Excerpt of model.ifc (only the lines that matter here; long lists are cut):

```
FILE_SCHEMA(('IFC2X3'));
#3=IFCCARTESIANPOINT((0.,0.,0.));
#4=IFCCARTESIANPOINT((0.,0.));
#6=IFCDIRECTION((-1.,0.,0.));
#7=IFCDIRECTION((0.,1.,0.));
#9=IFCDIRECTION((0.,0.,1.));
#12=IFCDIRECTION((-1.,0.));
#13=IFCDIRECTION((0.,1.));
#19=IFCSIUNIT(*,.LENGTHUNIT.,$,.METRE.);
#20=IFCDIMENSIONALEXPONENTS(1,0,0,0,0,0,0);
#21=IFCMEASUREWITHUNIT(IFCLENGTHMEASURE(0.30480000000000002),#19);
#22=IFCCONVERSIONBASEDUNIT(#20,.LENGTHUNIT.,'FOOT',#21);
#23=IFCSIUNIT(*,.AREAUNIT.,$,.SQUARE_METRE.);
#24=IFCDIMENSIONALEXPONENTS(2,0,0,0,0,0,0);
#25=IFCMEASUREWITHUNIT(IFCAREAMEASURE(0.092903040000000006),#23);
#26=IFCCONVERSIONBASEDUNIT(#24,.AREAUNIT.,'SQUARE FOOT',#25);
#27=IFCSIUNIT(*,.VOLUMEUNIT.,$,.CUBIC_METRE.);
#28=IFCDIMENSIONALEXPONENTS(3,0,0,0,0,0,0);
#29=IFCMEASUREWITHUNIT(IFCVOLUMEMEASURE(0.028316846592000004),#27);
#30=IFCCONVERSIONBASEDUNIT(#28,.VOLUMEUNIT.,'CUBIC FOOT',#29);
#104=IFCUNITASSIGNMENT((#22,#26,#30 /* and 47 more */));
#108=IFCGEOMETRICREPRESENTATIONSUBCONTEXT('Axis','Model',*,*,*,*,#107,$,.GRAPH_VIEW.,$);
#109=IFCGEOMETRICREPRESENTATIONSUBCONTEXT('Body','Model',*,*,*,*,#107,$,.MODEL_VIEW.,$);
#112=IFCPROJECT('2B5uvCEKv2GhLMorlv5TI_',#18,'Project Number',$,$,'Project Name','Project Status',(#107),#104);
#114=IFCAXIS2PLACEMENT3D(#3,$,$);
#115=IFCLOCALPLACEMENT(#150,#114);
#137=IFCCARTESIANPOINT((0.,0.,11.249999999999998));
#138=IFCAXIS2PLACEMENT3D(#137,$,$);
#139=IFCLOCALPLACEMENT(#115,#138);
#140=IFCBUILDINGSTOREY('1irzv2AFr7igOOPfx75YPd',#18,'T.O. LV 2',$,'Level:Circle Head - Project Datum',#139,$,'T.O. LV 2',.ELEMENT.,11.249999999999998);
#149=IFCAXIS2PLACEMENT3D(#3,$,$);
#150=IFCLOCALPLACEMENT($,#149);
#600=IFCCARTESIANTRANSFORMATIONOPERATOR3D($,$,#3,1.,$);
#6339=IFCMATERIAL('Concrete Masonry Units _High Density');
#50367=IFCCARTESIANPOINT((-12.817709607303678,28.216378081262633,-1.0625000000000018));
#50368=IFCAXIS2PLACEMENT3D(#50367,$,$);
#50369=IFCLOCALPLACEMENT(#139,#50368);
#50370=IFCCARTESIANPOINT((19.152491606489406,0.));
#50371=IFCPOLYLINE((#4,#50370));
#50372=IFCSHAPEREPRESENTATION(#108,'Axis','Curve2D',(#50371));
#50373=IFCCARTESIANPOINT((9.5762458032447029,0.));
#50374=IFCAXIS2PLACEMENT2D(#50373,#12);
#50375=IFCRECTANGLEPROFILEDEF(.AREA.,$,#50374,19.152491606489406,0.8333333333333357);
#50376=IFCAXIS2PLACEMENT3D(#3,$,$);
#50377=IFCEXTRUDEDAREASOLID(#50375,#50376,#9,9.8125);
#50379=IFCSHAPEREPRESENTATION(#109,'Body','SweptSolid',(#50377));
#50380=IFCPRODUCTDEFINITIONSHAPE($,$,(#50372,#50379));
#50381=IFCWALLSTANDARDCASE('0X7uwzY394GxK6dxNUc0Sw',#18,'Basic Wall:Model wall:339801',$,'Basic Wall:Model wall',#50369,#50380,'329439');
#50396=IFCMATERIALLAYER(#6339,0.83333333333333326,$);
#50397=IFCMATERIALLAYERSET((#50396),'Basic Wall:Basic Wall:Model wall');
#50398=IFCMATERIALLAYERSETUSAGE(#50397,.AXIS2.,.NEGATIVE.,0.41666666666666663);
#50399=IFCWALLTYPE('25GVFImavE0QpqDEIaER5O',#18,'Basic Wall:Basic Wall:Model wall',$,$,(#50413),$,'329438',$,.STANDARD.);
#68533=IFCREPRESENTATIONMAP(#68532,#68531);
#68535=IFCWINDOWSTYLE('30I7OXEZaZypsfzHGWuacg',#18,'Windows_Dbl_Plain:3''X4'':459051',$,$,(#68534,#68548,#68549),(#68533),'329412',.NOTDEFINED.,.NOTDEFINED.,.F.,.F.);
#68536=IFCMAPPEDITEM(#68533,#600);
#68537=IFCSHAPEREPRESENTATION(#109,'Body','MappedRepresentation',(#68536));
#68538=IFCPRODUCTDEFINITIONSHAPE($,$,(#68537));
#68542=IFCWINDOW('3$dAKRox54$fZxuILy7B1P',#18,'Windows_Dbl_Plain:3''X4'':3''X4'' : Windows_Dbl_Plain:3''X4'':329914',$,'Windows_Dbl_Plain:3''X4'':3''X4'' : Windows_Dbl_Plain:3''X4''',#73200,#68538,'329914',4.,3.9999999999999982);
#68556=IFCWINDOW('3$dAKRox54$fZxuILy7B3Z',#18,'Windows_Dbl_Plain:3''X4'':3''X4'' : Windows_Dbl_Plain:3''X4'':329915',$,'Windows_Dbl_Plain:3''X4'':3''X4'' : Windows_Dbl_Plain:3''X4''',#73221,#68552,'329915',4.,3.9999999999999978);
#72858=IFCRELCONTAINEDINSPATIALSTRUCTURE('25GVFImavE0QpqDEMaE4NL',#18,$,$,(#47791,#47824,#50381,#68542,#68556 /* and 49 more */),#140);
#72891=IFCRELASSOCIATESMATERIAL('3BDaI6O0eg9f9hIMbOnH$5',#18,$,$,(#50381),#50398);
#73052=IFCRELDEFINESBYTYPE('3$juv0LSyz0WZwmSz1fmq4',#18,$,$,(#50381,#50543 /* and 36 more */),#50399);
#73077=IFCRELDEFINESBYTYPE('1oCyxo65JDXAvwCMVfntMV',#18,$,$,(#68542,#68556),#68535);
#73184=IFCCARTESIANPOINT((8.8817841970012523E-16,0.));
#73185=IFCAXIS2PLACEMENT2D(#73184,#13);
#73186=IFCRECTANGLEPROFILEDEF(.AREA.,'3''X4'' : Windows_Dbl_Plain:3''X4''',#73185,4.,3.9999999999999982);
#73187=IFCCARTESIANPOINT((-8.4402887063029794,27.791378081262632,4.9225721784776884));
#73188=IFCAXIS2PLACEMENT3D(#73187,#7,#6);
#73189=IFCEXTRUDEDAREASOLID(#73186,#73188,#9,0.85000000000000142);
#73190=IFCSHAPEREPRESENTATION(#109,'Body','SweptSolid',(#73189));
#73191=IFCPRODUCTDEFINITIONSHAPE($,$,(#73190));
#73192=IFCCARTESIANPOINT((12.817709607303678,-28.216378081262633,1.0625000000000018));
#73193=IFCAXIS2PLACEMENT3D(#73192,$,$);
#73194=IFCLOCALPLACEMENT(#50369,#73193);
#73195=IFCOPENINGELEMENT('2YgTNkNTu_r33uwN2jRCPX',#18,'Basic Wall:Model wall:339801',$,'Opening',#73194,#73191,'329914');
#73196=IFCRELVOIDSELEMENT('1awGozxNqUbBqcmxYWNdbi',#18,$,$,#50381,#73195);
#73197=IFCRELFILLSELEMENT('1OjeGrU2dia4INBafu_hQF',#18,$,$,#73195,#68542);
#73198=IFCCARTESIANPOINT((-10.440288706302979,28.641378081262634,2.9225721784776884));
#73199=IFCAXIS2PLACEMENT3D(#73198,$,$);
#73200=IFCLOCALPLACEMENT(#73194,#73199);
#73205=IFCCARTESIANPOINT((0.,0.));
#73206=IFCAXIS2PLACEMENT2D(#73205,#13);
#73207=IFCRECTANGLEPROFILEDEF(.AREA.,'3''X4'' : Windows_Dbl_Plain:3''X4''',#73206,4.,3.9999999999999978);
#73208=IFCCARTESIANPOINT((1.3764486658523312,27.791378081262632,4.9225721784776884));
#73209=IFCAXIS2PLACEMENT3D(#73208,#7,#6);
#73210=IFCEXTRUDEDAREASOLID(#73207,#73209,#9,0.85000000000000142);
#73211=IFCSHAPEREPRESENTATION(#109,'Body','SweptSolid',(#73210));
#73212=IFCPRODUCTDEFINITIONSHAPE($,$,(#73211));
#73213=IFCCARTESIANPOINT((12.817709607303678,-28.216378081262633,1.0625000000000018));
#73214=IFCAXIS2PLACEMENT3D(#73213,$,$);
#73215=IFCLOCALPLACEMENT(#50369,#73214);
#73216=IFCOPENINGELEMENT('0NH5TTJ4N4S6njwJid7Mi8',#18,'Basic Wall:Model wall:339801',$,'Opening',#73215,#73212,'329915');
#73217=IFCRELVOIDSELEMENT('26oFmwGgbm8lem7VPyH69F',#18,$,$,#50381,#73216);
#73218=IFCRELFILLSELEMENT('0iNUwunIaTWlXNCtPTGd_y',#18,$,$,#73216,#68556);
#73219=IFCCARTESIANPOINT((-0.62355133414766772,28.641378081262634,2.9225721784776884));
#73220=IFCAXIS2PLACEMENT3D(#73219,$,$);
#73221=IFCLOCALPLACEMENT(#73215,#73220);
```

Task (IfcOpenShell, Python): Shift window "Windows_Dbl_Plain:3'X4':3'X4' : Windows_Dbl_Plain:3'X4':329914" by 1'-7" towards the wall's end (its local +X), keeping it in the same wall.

```python
import ifcopenshell
import ifcopenshell.api.geometry
import ifcopenshell.util.placement
import ifcopenshell.util.unit

model = ifcopenshell.open("model.ifc")
unit_scale = ifcopenshell.util.unit.calculate_unit_scale(model)

window = model.by_guid("3$dAKRox54$fZxuILy7B1P")
opening = window.FillsVoids[0].RelatingOpeningElement
wall = opening.VoidsElements[0].RelatingBuildingElement

wall_matrix = ifcopenshell.util.placement.get_local_placement(wall.ObjectPlacement)
shift = wall_matrix[:3, 0] * 19 * 0.0254 / unit_scale
before = ifcopenshell.util.placement.get_local_placement(window.ObjectPlacement)[:3, 3].copy()

# The window is placed relative to its opening, so it follows when the opening moves.
matrix = ifcopenshell.util.placement.get_local_placement(opening.ObjectPlacement)
matrix[:3, 3] += shift
ifcopenshell.api.geometry.edit_object_placement(
    model, product=opening, matrix=matrix, is_si=False, should_transform_children=True
)

after = ifcopenshell.util.placement.get_local_placement(window.ObjectPlacement)[:3, 3]
print("window moved by", (after - before).round(3) + 0.0)

model.write("model_updated.ifc")
```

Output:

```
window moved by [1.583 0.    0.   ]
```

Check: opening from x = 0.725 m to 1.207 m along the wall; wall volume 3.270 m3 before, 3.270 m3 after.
